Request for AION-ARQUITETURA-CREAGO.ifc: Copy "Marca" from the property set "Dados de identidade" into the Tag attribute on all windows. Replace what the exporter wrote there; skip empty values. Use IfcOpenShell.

First a look at what the model holds.

```python
import ifcopenshell
import ifcopenshell.util.element

model = ifcopenshell.open("AION-ARQUITETURA-CREAGO.ifc")
print(model.schema)
windows = model.by_type("IfcWindow")
print(len(windows), "windows")
for e in windows[:8]:
    source = ifcopenshell.util.element.get_pset(e, "Dados de identidade", "Marca")
    target = e.Tag
    print(e.id(), repr(source), repr(target), sep=" | ")
```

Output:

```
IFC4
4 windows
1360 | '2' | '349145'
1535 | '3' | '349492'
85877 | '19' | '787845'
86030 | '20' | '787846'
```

```python
import ifcopenshell
import ifcopenshell.util.element

model = ifcopenshell.open("AION-ARQUITETURA-CREAGO.ifc")

count = 0
for e in model.by_type("IfcWindow"):
    value = ifcopenshell.util.element.get_pset(e, "Dados de identidade", "Marca")
    current = e.Tag
    if not value or not value.strip() or current == value:
        continue
    e.Tag = value
    count += 1

print(count, "windows updated")

model.write("AION-ARQUITETURA-CREAGO_updated.ifc")
```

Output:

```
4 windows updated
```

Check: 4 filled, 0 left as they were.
